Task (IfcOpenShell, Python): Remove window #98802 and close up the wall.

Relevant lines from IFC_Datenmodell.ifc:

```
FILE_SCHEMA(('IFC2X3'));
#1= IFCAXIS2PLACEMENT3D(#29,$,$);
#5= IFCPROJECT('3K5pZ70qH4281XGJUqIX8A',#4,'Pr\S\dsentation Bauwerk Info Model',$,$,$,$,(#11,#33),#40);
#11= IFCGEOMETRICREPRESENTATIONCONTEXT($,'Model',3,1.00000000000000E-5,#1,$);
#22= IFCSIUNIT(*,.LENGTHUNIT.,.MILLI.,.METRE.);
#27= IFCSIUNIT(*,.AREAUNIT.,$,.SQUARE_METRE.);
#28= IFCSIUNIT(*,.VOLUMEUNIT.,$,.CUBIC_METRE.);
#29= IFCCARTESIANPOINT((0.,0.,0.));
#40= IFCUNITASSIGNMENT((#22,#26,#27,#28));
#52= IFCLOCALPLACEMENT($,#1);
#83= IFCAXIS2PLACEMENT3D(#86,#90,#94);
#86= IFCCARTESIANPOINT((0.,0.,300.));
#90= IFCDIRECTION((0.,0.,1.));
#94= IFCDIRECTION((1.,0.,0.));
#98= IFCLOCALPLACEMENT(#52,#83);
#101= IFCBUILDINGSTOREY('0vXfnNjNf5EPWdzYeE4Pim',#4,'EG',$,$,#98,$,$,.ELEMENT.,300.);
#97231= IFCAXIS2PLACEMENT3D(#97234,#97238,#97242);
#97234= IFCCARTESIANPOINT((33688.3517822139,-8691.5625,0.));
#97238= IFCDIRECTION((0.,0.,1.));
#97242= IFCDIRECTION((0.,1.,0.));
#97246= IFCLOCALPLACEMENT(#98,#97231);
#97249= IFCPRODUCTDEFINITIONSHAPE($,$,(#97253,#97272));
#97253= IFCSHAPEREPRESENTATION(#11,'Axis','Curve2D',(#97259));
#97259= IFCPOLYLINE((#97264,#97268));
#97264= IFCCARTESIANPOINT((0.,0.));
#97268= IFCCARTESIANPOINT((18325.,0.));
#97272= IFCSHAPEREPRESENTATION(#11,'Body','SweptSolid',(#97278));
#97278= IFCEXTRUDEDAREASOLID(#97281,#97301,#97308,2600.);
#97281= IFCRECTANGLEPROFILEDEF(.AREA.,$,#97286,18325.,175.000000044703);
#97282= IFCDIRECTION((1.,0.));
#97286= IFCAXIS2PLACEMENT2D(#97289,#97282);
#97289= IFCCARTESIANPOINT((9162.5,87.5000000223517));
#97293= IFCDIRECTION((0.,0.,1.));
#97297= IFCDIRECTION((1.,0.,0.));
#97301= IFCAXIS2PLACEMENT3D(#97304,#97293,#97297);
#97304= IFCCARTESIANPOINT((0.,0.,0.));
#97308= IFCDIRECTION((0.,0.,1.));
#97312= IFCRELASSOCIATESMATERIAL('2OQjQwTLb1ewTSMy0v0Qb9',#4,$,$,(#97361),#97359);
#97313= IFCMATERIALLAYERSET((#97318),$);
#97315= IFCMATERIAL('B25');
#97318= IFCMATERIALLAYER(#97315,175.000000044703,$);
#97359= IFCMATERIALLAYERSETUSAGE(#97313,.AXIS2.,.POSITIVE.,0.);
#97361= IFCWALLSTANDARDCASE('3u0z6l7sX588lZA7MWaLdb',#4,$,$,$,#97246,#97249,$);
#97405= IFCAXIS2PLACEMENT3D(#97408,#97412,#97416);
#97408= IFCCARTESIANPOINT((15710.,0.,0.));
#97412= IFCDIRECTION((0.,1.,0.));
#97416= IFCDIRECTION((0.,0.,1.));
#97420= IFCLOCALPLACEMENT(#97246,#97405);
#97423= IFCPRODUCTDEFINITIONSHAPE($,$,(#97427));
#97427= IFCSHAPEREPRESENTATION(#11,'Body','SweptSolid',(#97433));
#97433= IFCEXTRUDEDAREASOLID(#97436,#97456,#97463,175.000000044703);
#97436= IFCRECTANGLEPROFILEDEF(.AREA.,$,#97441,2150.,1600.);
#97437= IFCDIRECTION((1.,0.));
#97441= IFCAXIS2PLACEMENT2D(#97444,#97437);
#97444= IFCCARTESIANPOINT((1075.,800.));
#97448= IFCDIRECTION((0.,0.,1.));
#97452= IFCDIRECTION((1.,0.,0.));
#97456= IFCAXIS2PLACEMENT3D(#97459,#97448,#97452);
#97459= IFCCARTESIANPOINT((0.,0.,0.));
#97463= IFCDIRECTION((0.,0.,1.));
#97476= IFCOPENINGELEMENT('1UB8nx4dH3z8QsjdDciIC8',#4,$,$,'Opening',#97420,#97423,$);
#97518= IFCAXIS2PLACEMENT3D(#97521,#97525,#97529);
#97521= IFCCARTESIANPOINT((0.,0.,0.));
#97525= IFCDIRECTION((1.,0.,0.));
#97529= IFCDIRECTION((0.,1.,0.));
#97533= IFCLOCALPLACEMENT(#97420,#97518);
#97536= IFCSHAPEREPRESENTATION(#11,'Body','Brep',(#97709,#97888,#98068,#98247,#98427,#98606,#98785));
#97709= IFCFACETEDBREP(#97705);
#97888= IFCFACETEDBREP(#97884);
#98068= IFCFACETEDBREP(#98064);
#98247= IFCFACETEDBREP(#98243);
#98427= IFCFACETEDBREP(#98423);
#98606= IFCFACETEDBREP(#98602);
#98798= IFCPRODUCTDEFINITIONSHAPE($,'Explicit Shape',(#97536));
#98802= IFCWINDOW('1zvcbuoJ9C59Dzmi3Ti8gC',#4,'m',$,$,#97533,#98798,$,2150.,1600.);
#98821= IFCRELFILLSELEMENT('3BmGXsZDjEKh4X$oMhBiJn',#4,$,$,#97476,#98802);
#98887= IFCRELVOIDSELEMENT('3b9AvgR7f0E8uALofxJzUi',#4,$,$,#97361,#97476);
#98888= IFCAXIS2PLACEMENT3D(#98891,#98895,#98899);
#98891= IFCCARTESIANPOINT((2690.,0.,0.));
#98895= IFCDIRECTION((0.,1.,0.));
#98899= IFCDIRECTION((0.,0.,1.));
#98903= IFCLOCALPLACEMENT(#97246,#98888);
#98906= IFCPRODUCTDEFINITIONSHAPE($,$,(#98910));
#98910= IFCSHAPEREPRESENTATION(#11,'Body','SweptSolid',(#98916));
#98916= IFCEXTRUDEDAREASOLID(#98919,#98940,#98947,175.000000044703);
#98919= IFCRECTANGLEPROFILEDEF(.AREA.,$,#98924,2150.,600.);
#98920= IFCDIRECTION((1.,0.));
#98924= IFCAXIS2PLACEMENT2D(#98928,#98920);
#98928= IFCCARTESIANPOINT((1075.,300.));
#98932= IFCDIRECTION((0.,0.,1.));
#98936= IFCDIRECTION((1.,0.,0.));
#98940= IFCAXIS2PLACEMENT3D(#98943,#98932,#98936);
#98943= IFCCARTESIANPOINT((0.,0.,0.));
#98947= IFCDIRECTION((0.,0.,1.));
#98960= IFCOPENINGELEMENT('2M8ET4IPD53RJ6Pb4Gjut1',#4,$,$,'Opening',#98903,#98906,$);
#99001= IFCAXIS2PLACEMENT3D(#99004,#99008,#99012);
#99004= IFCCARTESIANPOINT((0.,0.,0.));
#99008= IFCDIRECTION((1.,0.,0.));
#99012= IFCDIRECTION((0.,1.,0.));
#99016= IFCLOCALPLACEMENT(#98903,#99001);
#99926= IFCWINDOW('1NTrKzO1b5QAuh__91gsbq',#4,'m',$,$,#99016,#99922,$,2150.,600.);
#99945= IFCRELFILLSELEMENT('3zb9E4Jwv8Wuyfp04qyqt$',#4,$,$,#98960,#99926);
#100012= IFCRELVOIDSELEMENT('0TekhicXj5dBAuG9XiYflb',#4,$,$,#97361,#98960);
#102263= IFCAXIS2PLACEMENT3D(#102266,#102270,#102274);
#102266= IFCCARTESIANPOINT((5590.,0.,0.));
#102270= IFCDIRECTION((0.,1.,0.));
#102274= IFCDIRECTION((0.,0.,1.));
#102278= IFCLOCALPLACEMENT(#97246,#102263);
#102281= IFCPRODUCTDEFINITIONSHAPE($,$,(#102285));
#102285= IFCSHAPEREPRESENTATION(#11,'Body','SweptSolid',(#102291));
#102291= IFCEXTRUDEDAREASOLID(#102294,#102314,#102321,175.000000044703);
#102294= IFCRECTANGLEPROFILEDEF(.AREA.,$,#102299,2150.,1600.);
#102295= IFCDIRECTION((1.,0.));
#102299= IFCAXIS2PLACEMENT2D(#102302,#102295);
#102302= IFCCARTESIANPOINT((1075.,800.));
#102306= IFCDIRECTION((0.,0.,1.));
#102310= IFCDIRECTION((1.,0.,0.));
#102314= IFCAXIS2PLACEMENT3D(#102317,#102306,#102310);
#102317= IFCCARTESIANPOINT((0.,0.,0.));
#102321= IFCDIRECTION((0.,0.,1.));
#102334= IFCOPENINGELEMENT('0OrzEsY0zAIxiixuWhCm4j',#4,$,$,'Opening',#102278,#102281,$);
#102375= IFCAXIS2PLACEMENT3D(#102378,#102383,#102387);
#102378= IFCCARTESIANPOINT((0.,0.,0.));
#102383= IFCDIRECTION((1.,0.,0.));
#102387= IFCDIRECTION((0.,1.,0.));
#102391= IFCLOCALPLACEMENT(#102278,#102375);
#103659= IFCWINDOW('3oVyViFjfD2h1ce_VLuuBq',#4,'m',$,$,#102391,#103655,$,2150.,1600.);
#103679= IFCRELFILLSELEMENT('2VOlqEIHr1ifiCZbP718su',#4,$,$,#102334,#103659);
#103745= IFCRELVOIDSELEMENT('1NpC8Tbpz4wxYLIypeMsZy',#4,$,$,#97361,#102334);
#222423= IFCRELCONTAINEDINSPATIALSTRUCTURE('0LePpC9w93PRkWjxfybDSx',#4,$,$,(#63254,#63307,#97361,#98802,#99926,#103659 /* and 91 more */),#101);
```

```python
import ifcopenshell
import ifcopenshell.api.feature
import ifcopenshell.api.root
import ifcopenshell.geom
import ifcopenshell.util.shape

model = ifcopenshell.open("IFC_Datenmodell.ifc")
settings = ifcopenshell.geom.settings()


def volume(element):
    """Net volume in cubic metres, openings subtracted."""
    shape = ifcopenshell.geom.create_shape(settings, element)
    return ifcopenshell.util.shape.get_volume(shape.geometry)


window = model.by_guid("1zvcbuoJ9C59Dzmi3Ti8gC")
opening = window.FillsVoids[0].RelatingOpeningElement
wall = opening.VoidsElements[0].RelatingBuildingElement
before = volume(wall)

ifcopenshell.api.root.remove_product(model, product=window)
ifcopenshell.api.feature.remove_feature(model, feature=opening)

after = volume(wall)

print(f"wall volume {before:.3f} -> {after:.3f} m3")

model.write("IFC_Datenmodell_v2.ifc")
```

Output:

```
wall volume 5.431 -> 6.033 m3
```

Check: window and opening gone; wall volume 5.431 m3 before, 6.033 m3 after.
